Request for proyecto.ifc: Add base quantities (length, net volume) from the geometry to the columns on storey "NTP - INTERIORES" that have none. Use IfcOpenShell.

First a look at what the model holds.

```python
import ifcopenshell
import ifcopenshell.util.element
import ifcopenshell.util.unit

model = ifcopenshell.open("proyecto.ifc")
print(model.schema)
for unit_type in ("LENGTHUNIT", "AREAUNIT", "VOLUMEUNIT"):
    print(unit_type, ifcopenshell.util.unit.calculate_unit_scale(model, unit_type))
storey = next(s for s in model.by_type("IfcBuildingStorey") if s.Name == "NTP - INTERIORES")
columns = [e for e in ifcopenshell.util.element.get_decomposition(storey) if e.is_a("IfcColumn")]
for e in sorted(columns, key=lambda e: e.id()):
    print(e.id(), e.is_a(), e.Name, list(ifcopenshell.util.element.get_psets(e, qtos_only=True)), sep=" | ")
```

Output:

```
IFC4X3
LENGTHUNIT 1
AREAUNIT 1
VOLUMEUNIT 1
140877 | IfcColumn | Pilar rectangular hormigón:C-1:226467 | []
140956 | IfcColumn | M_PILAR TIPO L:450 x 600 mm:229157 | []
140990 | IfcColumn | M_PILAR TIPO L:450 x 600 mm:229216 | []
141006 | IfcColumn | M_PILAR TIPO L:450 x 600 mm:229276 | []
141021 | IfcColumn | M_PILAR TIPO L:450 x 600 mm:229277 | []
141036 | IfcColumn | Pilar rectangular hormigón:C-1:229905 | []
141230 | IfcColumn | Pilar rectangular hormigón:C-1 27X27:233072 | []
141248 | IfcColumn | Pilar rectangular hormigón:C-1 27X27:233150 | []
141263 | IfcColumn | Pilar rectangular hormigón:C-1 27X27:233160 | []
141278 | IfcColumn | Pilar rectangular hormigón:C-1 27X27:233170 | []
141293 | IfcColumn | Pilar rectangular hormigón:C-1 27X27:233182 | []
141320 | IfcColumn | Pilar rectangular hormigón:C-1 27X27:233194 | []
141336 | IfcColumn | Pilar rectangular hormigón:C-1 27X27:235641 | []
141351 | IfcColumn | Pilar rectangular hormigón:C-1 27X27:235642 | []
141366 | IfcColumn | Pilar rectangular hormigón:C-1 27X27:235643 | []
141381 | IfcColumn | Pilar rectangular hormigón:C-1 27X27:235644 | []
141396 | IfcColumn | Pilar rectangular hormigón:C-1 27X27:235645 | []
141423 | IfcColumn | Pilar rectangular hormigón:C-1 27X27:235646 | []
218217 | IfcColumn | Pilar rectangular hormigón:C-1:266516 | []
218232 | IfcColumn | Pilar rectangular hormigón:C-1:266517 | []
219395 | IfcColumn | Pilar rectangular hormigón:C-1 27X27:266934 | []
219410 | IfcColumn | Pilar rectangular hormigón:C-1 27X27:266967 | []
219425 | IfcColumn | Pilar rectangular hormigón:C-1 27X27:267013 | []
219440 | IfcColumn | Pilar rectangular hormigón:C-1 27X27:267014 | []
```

```python
import ifcopenshell
import ifcopenshell.api.pset
import ifcopenshell.geom
import ifcopenshell.util.element
import ifcopenshell.util.shape
import ifcopenshell.util.unit

model = ifcopenshell.open("proyecto.ifc")
unit_scale = ifcopenshell.util.unit.calculate_unit_scale(model)
volume_scale = ifcopenshell.util.unit.calculate_unit_scale(model, "VOLUMEUNIT")
settings = ifcopenshell.geom.settings()

storey = next(s for s in model.by_type("IfcBuildingStorey") if s.Name == "NTP - INTERIORES")
columns = [e for e in ifcopenshell.util.element.get_decomposition(storey) if e.is_a("IfcColumn")]

for e in sorted(columns, key=lambda e: e.id()):
    if ifcopenshell.util.element.get_psets(e, qtos_only=True, should_inherit=False):
        continue
    # Geometry comes back in metres, in the element's own axes.
    shape = ifcopenshell.geom.create_shape(settings, e)
    values = {
        "Length": ifcopenshell.util.shape.get_z(shape.geometry) / unit_scale,
        "NetVolume": ifcopenshell.util.shape.get_volume(shape.geometry) / volume_scale,
    }
    qto = ifcopenshell.api.pset.add_qto(model, product=e, name="Qto_ColumnBaseQuantities")
    ifcopenshell.api.pset.edit_qto(model, qto=qto, properties=values)
    print(e.id(), {k: round(v, 3) for k, v in values.items()})

model.write("proyecto_updated.ifc")
```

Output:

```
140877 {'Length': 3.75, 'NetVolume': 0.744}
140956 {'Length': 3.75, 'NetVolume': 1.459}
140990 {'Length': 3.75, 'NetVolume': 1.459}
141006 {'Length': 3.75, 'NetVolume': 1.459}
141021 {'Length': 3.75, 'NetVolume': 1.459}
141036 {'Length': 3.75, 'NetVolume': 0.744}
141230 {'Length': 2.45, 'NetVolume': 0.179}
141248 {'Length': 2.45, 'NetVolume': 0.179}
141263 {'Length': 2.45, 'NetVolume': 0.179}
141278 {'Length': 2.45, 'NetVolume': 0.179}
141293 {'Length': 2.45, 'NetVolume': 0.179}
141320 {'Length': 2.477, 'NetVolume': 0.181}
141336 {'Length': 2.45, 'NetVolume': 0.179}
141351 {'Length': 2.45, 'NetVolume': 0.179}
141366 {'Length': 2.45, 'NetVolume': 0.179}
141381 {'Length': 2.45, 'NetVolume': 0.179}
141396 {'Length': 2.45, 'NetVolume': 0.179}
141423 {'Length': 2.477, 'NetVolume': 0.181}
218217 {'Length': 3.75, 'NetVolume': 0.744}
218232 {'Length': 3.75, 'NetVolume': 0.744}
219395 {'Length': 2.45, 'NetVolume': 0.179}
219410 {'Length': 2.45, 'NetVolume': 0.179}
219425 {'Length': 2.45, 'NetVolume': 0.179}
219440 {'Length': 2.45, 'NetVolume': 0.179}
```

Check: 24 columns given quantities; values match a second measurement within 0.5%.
